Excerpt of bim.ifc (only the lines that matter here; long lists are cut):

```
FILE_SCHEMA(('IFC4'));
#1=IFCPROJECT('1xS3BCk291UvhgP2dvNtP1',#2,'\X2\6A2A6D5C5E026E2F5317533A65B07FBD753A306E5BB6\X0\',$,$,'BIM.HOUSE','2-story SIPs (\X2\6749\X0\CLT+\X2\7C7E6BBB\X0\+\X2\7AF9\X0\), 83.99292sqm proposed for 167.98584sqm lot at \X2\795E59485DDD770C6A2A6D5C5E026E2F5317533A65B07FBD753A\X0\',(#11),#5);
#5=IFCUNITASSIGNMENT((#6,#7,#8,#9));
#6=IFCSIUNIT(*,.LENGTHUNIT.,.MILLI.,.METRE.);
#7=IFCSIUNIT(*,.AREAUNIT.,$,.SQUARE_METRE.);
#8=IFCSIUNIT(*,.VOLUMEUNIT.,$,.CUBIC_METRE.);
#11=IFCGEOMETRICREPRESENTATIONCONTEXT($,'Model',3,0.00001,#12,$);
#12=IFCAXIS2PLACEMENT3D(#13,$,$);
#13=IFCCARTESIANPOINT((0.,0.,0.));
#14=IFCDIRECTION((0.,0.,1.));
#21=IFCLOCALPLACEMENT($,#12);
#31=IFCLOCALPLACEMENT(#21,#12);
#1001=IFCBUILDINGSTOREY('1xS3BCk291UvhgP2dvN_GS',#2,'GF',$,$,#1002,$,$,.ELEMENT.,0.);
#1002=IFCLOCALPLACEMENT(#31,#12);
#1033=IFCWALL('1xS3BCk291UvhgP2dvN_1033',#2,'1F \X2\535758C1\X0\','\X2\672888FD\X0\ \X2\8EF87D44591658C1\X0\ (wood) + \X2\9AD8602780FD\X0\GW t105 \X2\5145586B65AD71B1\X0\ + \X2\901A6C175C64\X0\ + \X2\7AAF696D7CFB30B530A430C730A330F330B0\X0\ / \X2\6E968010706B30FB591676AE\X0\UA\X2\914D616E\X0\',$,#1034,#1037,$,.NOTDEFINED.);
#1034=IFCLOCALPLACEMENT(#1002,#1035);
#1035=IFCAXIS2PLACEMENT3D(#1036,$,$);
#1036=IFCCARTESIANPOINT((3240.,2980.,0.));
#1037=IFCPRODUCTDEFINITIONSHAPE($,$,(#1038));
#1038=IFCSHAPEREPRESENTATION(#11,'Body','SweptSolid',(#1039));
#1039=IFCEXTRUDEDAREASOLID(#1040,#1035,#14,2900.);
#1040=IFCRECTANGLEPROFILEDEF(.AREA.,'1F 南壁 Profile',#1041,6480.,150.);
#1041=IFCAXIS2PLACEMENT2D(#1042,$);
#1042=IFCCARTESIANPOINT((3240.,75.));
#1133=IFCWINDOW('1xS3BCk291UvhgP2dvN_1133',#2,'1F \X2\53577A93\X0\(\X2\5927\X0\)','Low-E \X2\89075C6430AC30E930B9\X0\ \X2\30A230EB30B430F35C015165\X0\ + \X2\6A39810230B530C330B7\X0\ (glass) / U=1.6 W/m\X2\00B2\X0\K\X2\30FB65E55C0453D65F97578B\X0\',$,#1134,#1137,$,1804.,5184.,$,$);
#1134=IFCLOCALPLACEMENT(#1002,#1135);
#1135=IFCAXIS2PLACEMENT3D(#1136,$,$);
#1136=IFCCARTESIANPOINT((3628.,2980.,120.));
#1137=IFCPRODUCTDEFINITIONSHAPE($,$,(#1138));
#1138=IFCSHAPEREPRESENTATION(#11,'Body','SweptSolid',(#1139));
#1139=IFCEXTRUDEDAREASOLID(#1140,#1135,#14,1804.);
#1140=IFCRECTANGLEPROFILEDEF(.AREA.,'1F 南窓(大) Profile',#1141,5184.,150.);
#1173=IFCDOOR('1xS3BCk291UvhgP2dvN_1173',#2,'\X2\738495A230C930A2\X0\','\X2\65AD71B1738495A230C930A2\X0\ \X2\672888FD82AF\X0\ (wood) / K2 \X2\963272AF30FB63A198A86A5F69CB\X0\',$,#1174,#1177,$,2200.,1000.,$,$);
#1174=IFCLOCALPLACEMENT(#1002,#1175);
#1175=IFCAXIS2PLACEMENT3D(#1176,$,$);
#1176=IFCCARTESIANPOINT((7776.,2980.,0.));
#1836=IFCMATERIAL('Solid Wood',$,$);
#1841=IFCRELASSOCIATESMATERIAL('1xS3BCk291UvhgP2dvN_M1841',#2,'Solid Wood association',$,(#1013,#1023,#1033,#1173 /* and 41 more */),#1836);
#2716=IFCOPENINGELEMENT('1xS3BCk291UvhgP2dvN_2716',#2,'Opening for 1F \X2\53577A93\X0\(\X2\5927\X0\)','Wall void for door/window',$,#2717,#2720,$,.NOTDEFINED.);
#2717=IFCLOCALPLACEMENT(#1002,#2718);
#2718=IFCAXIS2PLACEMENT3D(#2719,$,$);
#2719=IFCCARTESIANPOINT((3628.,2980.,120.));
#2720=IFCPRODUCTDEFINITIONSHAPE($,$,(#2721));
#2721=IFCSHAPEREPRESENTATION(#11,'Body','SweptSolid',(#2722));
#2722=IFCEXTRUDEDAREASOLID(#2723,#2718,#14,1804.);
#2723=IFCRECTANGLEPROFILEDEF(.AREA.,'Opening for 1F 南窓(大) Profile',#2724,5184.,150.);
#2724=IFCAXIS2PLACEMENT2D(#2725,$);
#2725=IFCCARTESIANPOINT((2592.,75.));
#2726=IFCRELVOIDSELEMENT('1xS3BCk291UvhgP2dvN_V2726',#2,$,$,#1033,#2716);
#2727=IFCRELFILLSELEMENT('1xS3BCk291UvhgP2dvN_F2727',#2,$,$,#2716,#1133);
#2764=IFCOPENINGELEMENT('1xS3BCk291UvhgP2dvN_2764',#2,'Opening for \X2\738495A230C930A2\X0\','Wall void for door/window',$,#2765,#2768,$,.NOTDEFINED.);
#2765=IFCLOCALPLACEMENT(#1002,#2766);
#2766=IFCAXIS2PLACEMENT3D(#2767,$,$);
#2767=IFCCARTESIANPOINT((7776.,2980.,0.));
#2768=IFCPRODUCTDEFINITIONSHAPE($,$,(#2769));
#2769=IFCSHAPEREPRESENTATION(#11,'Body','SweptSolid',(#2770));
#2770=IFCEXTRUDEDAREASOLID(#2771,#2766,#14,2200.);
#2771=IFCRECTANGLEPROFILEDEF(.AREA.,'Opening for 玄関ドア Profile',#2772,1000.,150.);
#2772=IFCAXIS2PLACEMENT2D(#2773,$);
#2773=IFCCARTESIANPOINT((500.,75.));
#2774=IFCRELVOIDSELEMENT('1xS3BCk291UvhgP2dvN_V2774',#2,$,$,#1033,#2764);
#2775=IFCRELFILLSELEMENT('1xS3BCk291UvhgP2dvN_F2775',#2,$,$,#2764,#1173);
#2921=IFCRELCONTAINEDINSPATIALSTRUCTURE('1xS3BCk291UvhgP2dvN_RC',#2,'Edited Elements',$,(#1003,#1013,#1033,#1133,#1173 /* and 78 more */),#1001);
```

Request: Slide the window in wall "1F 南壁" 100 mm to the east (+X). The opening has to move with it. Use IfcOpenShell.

```python
import ifcopenshell
import ifcopenshell.api.geometry
import ifcopenshell.util.placement

model = ifcopenshell.open("bim.ifc")

window = model.by_guid("1xS3BCk291UvhgP2dvN_1133")
opening = window.FillsVoids[0].RelatingOpeningElement
wall = opening.VoidsElements[0].RelatingBuildingElement

wall_matrix = ifcopenshell.util.placement.get_local_placement(wall.ObjectPlacement)
shift = wall_matrix[:3, 0] * 100.0
before = ifcopenshell.util.placement.get_local_placement(window.ObjectPlacement)[:3, 3].copy()

# The window is not placed relative to its opening, so move both.
for product in (opening, window):
    matrix = ifcopenshell.util.placement.get_local_placement(product.ObjectPlacement)
    matrix[:3, 3] += shift
    ifcopenshell.api.geometry.edit_object_placement(model, product=product, matrix=matrix, is_si=False)

after = ifcopenshell.util.placement.get_local_placement(window.ObjectPlacement)[:3, 3]
print("window moved by", (after - before).round(3) + 0.0)

model.write("bim_rev.ifc")
```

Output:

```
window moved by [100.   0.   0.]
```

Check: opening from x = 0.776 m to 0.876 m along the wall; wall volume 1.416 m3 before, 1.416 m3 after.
